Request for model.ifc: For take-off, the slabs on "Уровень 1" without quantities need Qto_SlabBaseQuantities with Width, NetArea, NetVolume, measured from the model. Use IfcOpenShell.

First a look at what the model holds.

```python
import ifcopenshell
import ifcopenshell.util.element
import ifcopenshell.util.unit

model = ifcopenshell.open("model.ifc")
print(model.schema)
for unit_type in ("LENGTHUNIT", "AREAUNIT", "VOLUMEUNIT"):
    print(unit_type, ifcopenshell.util.unit.calculate_unit_scale(model, unit_type))
storey = next(s for s in model.by_type("IfcBuildingStorey") if s.Name == "Уровень 1")
slabs = [e for e in ifcopenshell.util.element.get_decomposition(storey) if e.is_a("IfcSlab")]
for e in sorted(slabs, key=lambda e: e.id()):
    print(e.id(), e.is_a(), e.Name, list(ifcopenshell.util.element.get_psets(e, qtos_only=True)), sep=" | ")
```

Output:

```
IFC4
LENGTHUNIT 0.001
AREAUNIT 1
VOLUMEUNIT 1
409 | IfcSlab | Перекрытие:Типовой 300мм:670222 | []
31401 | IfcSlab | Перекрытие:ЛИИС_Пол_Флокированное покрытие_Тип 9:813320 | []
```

```python
import ifcopenshell
import ifcopenshell.api.pset
import ifcopenshell.geom
import ifcopenshell.util.element
import ifcopenshell.util.shape
import ifcopenshell.util.unit

model = ifcopenshell.open("model.ifc")
unit_scale = ifcopenshell.util.unit.calculate_unit_scale(model)
area_scale = ifcopenshell.util.unit.calculate_unit_scale(model, "AREAUNIT")
volume_scale = ifcopenshell.util.unit.calculate_unit_scale(model, "VOLUMEUNIT")
settings = ifcopenshell.geom.settings()

storey = next(s for s in model.by_type("IfcBuildingStorey") if s.Name == "Уровень 1")
slabs = [e for e in ifcopenshell.util.element.get_decomposition(storey) if e.is_a("IfcSlab")]

for e in sorted(slabs, key=lambda e: e.id()):
    if ifcopenshell.util.element.get_psets(e, qtos_only=True, should_inherit=False):
        continue
    # Geometry comes back in metres, in the element's own axes.
    shape = ifcopenshell.geom.create_shape(settings, e)
    values = {
        "Width": ifcopenshell.util.shape.get_z(shape.geometry) / unit_scale,
        "NetArea": ifcopenshell.util.shape.get_footprint_area(shape.geometry) / area_scale,
        "NetVolume": ifcopenshell.util.shape.get_volume(shape.geometry) / volume_scale,
    }
    qto = ifcopenshell.api.pset.add_qto(model, product=e, name="Qto_SlabBaseQuantities")
    ifcopenshell.api.pset.edit_qto(model, qto=qto, properties=values)
    print(e.id(), {k: round(v, 3) for k, v in values.items()})

model.write("model-out.ifc")
```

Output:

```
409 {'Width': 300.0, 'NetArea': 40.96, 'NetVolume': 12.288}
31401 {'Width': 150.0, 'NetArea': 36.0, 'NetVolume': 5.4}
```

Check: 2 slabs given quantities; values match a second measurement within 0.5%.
